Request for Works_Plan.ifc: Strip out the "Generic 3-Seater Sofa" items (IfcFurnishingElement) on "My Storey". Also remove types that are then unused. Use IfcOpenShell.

First a look at what the model holds.

```python
import ifcopenshell
import ifcopenshell.util.element

model = ifcopenshell.open("Works_Plan.ifc")
print(model.schema)
storey = next(s for s in model.by_type("IfcBuildingStorey") if s.Name == "My Storey")
furniture = [e for e in ifcopenshell.util.element.get_decomposition(storey) if e.is_a("IfcFurnishingElement")]
seen = {}
for e in furniture:
    element_type = ifcopenshell.util.element.get_type(e)
    name = element_type.Name if element_type not in (None, e) else None
    seen[name] = seen.get(name, 0) + 1
for name, count in sorted(seen.items(), key=str):
    print(count, "x", name)
```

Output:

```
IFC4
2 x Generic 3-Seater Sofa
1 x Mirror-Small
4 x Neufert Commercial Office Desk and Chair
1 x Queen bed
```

```python
import ifcopenshell
import ifcopenshell.api.root
import ifcopenshell.util.element

model = ifcopenshell.open("Works_Plan.ifc")

storey = next(s for s in model.by_type("IfcBuildingStorey") if s.Name == "My Storey")
furniture = [e for e in ifcopenshell.util.element.get_decomposition(storey) if e.is_a("IfcFurnishingElement")]
targets = [e for e in furniture if (t := ifcopenshell.util.element.get_type(e)) not in (None, e) and t.Name == "Generic 3-Seater Sofa"]
types = {ifcopenshell.util.element.get_type(e) for e in targets} - {None, *targets}

for e in targets:
    ifcopenshell.api.root.remove_product(model, product=e)
print(len(targets), "removed")

unused = [t for t in types if not ifcopenshell.util.element.get_types(t)]
for t in unused:
    ifcopenshell.api.root.remove_product(model, product=t)
print(len(unused), "unused types removed")

model.write("Works_Plan_updated.ifc")
```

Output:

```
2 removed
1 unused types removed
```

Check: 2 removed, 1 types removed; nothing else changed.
